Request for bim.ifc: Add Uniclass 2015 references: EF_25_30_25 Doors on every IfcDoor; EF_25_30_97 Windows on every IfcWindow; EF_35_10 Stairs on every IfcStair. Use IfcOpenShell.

First a look at what the model holds.

```python
import ifcopenshell

model = ifcopenshell.open("bim.ifc")
print(model.schema)
print("classifications:", [c.Name for c in model.by_type("IfcClassification")])
for ifc_class in ("IfcDoor", "IfcRoof", "IfcStair", "IfcWall", "IfcWindow"):
    print(ifc_class, len(model.by_type(ifc_class)))
```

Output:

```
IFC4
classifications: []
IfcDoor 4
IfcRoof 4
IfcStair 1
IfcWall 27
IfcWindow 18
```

```python
import ifcopenshell
import ifcopenshell.api.classification

model = ifcopenshell.open("bim.ifc")

system = ifcopenshell.api.classification.add_classification(model, classification="Uniclass 2015")

codes = {
    "IfcDoor": ("EF_25_30_25", "Doors"),
    "IfcWindow": ("EF_25_30_97", "Windows"),
    "IfcStair": ("EF_35_10", "Stairs"),
}
for ifc_class, (code, name) in codes.items():
    products = model.by_type(ifc_class)
    ifcopenshell.api.classification.add_reference(
        model, products=products, classification=system, identification=code, name=name
    )
    print(code, len(products))

model.write("bim_rev.ifc")
```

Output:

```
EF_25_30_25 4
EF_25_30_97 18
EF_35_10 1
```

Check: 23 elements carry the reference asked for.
